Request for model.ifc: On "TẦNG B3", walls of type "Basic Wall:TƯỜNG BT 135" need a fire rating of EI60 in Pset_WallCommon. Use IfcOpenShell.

First a look at what the model holds.

```python
import ifcopenshell
import ifcopenshell.util.element

model = ifcopenshell.open("model.ifc")
print(model.schema)
storey = next(s for s in model.by_type("IfcBuildingStorey") if s.Name == "TẦNG B3")
walls = [e for e in ifcopenshell.util.element.get_decomposition(storey) if e.is_a("IfcWall")]
seen = {}
for e in walls:
    element_type = ifcopenshell.util.element.get_type(e)
    key = (element_type.Name if element_type != e and element_type else None, ifcopenshell.util.element.get_pset(e, "Pset_WallCommon", "FireRating"))
    seen[key] = seen.get(key, 0) + 1
for (name, value), count in sorted(seen.items(), key=str):
    print(count, "x", name, "|", value)
```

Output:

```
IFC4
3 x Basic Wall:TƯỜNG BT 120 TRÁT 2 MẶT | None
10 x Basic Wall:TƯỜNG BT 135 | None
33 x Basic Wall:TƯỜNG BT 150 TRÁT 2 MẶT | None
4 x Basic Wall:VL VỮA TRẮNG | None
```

```python
import ifcopenshell
import ifcopenshell.api.pset
import ifcopenshell.util.element

model = ifcopenshell.open("model.ifc")

storey = next(s for s in model.by_type("IfcBuildingStorey") if s.Name == "TẦNG B3")
walls = [e for e in ifcopenshell.util.element.get_decomposition(storey) if e.is_a("IfcWall")]

count = 0
for e in walls:
    element_type = ifcopenshell.util.element.get_type(e)
    if element_type in (None, e) or element_type.Name != "Basic Wall:TƯỜNG BT 135":
        continue
    # add_pset returns the element's existing set when there is one.
    pset = ifcopenshell.api.pset.add_pset(model, product=e, name="Pset_WallCommon")
    ifcopenshell.api.pset.edit_pset(model, pset=pset, properties={"FireRating": "EI60"})
    count += 1

print(count, "walls updated")

model.write("model_edited.ifc")
```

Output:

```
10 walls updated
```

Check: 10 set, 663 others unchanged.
